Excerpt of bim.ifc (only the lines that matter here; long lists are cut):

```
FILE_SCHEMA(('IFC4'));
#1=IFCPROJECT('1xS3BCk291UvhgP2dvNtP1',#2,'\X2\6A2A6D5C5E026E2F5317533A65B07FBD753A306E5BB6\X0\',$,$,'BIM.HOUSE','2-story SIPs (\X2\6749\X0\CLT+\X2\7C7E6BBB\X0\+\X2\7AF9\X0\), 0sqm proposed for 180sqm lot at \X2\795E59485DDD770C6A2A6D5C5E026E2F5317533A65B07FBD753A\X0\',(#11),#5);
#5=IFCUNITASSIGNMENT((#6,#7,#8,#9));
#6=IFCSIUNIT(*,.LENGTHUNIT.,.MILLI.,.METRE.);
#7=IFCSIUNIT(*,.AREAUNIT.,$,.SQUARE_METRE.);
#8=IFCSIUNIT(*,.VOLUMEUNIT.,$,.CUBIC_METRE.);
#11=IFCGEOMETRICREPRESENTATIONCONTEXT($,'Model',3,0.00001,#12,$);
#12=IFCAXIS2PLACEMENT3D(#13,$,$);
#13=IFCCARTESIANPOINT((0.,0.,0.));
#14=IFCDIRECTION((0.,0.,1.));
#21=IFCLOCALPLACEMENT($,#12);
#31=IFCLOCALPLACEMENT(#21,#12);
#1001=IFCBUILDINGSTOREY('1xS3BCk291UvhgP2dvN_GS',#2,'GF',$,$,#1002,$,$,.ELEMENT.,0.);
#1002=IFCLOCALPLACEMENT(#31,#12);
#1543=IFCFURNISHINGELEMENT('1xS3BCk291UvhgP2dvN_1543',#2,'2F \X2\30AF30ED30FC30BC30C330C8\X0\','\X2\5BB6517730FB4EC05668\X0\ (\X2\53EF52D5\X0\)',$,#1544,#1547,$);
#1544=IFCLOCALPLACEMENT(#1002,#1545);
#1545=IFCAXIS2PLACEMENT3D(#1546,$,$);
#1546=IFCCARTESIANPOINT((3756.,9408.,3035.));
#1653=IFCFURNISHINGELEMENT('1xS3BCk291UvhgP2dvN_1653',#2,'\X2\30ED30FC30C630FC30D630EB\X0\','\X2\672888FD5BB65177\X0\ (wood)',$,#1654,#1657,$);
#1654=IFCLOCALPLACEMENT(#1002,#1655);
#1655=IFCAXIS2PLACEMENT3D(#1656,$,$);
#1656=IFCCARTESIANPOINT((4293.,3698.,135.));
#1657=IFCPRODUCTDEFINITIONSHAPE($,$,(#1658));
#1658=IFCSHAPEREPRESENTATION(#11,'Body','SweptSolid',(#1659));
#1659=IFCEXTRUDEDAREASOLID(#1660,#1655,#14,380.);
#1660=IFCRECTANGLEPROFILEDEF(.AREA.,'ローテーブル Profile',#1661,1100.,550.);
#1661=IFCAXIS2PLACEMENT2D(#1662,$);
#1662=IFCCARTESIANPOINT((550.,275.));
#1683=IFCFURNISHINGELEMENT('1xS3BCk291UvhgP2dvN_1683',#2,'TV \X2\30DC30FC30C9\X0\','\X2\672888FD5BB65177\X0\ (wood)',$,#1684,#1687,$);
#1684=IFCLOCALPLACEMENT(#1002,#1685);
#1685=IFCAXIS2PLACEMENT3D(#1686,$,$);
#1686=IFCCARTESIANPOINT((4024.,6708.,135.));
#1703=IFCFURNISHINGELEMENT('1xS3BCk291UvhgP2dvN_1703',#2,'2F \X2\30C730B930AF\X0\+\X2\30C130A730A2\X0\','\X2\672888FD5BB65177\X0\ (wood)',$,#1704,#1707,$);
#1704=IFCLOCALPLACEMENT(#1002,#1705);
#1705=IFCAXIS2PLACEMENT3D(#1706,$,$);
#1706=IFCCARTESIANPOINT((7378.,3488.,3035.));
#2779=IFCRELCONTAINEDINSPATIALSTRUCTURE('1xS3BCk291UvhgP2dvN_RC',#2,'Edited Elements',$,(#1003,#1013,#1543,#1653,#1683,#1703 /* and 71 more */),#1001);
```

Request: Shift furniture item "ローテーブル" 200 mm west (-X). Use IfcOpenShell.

```python
import ifcopenshell
import ifcopenshell.api.geometry
import ifcopenshell.util.placement
import ifcopenshell.util.unit

model = ifcopenshell.open("bim.ifc")
unit_scale = ifcopenshell.util.unit.calculate_unit_scale(model)

item = model.by_guid("1xS3BCk291UvhgP2dvN_1653")
matrix = ifcopenshell.util.placement.get_local_placement(item.ObjectPlacement)
matrix[0, 3] -= 0.2 / unit_scale
ifcopenshell.api.geometry.edit_object_placement(model, product=item, matrix=matrix, is_si=False)

print(ifcopenshell.util.placement.get_local_placement(item.ObjectPlacement).round(3) + 0.0)

model.write("bim_updated.ifc")
```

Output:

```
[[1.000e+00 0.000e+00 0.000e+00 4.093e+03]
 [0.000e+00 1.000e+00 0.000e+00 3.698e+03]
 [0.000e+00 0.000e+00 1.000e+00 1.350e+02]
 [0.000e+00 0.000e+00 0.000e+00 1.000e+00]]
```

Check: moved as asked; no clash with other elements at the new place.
